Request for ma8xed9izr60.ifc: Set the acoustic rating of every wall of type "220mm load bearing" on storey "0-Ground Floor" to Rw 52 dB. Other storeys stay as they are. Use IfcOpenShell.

First a look at what the model holds.

```python
import ifcopenshell
import ifcopenshell.util.element

model = ifcopenshell.open("ma8xed9izr60.ifc")
print(model.schema)
storey = next(s for s in model.by_type("IfcBuildingStorey") if s.Name == "0-Ground Floor")
walls = [e for e in ifcopenshell.util.element.get_decomposition(storey) if e.is_a("IfcWall")]
seen = {}
for e in walls:
    element_type = ifcopenshell.util.element.get_type(e)
    key = (element_type.Name if element_type != e and element_type else None, ifcopenshell.util.element.get_pset(e, "Pset_WallCommon", "AcousticRating"))
    seen[key] = seen.get(key, 0) + 1
for (name, value), count in sorted(seen.items(), key=str):
    print(count, "x", name, "|", value)
```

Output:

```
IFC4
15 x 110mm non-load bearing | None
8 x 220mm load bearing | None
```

```python
import ifcopenshell
import ifcopenshell.api.pset
import ifcopenshell.util.element

model = ifcopenshell.open("ma8xed9izr60.ifc")

storey = next(s for s in model.by_type("IfcBuildingStorey") if s.Name == "0-Ground Floor")
walls = [e for e in ifcopenshell.util.element.get_decomposition(storey) if e.is_a("IfcWall")]

count = 0
for e in walls:
    element_type = ifcopenshell.util.element.get_type(e)
    if element_type in (None, e) or element_type.Name != "220mm load bearing":
        continue
    # add_pset returns the element's existing set when there is one.
    pset = ifcopenshell.api.pset.add_pset(model, product=e, name="Pset_WallCommon")
    ifcopenshell.api.pset.edit_pset(model, pset=pset, properties={"AcousticRating": "Rw 52 dB"})
    count += 1

print(count, "walls updated")

model.write("ma8xed9izr60_updated.ifc")
```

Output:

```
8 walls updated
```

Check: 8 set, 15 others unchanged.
